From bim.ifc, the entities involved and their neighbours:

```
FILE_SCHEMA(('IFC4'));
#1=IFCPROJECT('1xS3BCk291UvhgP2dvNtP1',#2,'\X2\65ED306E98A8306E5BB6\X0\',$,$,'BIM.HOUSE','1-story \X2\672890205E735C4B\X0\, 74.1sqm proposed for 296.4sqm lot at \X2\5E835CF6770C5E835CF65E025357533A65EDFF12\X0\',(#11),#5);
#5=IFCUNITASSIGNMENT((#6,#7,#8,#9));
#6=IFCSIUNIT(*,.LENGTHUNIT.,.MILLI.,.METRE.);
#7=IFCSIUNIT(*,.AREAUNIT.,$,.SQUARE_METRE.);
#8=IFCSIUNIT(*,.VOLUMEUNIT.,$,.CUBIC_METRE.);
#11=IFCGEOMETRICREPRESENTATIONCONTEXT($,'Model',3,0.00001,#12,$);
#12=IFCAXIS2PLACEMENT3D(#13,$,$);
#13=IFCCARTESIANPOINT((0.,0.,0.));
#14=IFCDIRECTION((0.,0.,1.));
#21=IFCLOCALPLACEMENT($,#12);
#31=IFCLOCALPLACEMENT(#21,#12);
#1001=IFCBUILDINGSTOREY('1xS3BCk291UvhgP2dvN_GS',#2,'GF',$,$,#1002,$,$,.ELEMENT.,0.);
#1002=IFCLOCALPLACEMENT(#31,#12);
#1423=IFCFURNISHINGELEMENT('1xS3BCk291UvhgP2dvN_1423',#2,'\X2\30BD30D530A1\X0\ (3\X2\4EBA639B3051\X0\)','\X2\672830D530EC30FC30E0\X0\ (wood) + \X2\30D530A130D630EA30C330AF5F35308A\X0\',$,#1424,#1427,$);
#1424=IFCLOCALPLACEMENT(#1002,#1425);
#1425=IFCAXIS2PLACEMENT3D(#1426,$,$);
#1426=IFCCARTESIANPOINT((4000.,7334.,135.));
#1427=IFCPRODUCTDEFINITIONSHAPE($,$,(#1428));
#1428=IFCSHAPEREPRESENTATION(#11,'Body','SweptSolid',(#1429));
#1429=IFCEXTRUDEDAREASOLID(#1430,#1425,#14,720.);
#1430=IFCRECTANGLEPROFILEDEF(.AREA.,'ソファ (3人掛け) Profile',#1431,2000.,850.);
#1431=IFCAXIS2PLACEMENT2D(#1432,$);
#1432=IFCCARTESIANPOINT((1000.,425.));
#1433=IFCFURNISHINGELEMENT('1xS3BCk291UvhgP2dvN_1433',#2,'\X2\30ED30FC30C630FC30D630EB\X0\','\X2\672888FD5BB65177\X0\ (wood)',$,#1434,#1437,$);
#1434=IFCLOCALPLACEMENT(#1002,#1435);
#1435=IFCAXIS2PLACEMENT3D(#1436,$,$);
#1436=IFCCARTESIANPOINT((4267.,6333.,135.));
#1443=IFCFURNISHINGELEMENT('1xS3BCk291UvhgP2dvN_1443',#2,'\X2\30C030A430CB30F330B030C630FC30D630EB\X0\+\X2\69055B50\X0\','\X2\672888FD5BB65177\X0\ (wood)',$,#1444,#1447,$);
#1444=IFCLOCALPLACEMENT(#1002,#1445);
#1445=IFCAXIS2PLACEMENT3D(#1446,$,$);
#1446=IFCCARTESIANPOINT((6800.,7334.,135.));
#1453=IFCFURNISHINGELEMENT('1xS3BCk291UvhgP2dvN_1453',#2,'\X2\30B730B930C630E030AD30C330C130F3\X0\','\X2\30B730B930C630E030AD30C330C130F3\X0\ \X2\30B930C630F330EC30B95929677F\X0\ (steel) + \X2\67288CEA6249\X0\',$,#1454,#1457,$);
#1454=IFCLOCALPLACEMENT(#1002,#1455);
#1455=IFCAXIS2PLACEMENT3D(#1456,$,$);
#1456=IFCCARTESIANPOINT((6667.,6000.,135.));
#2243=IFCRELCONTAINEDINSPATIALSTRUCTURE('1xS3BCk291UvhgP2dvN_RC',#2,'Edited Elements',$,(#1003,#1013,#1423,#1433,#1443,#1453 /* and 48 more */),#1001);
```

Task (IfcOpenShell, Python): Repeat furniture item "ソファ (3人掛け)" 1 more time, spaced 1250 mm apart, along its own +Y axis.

```python
import ifcopenshell
import ifcopenshell.api.geometry
import ifcopenshell.api.root
import ifcopenshell.util.element
import ifcopenshell.util.placement
import ifcopenshell.util.unit

model = ifcopenshell.open("bim.ifc")
unit_scale = ifcopenshell.util.unit.calculate_unit_scale(model)


def reuse_history(source, copy):
    """copy_class also copies each property set's owner history, people and application; keep the originals."""
    for rel in copy.IsDefinedBy:
        if rel.is_a("IfcRelDefinesByProperties") and (history := rel.RelatingPropertyDefinition.OwnerHistory):
            rel.RelatingPropertyDefinition.OwnerHistory = source.OwnerHistory
            ifcopenshell.util.element.remove_deep2(model, history)


source = model.by_guid("1xS3BCk291UvhgP2dvN_1423")
base = ifcopenshell.util.placement.get_local_placement(source.ObjectPlacement)
step = base[:3, 1] * 1.25 / unit_scale

for i in range(1, 2):
    copy = ifcopenshell.api.root.copy_class(model, product=source)
    copy.Representation = ifcopenshell.util.element.copy_deep(
        model, source.Representation, exclude=["IfcGeometricRepresentationContext", "IfcRepresentationMap"]
    )
    reuse_history(source, copy)
    matrix = base.copy()
    matrix[:3, 3] += i * step
    print("added at", matrix[:3, 3].round(3) + 0.0)
    ifcopenshell.api.geometry.edit_object_placement(model, product=copy, matrix=matrix, is_si=False)

model.write("bim_updated.ifc")
```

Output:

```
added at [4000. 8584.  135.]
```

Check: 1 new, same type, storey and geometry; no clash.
